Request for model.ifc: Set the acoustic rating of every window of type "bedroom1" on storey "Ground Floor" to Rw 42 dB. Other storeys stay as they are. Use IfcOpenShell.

First a look at what the model holds.

```python
import ifcopenshell
import ifcopenshell.util.element

model = ifcopenshell.open("model.ifc")
print(model.schema)
storey = next(s for s in model.by_type("IfcBuildingStorey") if s.Name == "Ground Floor")
windows = [e for e in ifcopenshell.util.element.get_decomposition(storey) if e.is_a("IfcWindow")]
seen = {}
for e in windows:
    element_type = ifcopenshell.util.element.get_type(e)
    key = (element_type.Name if element_type != e and element_type else None, ifcopenshell.util.element.get_pset(e, "Pset_WindowCommon", "AcousticRating"))
    seen[key] = seen.get(key, 0) + 1
for (name, value), count in sorted(seen.items(), key=str):
    print(count, "x", name, "|", value)
```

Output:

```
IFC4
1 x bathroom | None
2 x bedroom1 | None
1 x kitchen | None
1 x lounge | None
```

```python
import ifcopenshell
import ifcopenshell.api.pset
import ifcopenshell.util.element

model = ifcopenshell.open("model.ifc")

storey = next(s for s in model.by_type("IfcBuildingStorey") if s.Name == "Ground Floor")
windows = [e for e in ifcopenshell.util.element.get_decomposition(storey) if e.is_a("IfcWindow")]

count = 0
for e in windows:
    element_type = ifcopenshell.util.element.get_type(e)
    if element_type in (None, e) or element_type.Name != "bedroom1":
        continue
    # add_pset returns the element's existing set when there is one.
    pset = ifcopenshell.api.pset.add_pset(model, product=e, name="Pset_WindowCommon")
    ifcopenshell.api.pset.edit_pset(model, pset=pset, properties={"AcousticRating": "Rw 42 dB"})
    count += 1

print(count, "windows updated")

model.write("model_edited.ifc")
```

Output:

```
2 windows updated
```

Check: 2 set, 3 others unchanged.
